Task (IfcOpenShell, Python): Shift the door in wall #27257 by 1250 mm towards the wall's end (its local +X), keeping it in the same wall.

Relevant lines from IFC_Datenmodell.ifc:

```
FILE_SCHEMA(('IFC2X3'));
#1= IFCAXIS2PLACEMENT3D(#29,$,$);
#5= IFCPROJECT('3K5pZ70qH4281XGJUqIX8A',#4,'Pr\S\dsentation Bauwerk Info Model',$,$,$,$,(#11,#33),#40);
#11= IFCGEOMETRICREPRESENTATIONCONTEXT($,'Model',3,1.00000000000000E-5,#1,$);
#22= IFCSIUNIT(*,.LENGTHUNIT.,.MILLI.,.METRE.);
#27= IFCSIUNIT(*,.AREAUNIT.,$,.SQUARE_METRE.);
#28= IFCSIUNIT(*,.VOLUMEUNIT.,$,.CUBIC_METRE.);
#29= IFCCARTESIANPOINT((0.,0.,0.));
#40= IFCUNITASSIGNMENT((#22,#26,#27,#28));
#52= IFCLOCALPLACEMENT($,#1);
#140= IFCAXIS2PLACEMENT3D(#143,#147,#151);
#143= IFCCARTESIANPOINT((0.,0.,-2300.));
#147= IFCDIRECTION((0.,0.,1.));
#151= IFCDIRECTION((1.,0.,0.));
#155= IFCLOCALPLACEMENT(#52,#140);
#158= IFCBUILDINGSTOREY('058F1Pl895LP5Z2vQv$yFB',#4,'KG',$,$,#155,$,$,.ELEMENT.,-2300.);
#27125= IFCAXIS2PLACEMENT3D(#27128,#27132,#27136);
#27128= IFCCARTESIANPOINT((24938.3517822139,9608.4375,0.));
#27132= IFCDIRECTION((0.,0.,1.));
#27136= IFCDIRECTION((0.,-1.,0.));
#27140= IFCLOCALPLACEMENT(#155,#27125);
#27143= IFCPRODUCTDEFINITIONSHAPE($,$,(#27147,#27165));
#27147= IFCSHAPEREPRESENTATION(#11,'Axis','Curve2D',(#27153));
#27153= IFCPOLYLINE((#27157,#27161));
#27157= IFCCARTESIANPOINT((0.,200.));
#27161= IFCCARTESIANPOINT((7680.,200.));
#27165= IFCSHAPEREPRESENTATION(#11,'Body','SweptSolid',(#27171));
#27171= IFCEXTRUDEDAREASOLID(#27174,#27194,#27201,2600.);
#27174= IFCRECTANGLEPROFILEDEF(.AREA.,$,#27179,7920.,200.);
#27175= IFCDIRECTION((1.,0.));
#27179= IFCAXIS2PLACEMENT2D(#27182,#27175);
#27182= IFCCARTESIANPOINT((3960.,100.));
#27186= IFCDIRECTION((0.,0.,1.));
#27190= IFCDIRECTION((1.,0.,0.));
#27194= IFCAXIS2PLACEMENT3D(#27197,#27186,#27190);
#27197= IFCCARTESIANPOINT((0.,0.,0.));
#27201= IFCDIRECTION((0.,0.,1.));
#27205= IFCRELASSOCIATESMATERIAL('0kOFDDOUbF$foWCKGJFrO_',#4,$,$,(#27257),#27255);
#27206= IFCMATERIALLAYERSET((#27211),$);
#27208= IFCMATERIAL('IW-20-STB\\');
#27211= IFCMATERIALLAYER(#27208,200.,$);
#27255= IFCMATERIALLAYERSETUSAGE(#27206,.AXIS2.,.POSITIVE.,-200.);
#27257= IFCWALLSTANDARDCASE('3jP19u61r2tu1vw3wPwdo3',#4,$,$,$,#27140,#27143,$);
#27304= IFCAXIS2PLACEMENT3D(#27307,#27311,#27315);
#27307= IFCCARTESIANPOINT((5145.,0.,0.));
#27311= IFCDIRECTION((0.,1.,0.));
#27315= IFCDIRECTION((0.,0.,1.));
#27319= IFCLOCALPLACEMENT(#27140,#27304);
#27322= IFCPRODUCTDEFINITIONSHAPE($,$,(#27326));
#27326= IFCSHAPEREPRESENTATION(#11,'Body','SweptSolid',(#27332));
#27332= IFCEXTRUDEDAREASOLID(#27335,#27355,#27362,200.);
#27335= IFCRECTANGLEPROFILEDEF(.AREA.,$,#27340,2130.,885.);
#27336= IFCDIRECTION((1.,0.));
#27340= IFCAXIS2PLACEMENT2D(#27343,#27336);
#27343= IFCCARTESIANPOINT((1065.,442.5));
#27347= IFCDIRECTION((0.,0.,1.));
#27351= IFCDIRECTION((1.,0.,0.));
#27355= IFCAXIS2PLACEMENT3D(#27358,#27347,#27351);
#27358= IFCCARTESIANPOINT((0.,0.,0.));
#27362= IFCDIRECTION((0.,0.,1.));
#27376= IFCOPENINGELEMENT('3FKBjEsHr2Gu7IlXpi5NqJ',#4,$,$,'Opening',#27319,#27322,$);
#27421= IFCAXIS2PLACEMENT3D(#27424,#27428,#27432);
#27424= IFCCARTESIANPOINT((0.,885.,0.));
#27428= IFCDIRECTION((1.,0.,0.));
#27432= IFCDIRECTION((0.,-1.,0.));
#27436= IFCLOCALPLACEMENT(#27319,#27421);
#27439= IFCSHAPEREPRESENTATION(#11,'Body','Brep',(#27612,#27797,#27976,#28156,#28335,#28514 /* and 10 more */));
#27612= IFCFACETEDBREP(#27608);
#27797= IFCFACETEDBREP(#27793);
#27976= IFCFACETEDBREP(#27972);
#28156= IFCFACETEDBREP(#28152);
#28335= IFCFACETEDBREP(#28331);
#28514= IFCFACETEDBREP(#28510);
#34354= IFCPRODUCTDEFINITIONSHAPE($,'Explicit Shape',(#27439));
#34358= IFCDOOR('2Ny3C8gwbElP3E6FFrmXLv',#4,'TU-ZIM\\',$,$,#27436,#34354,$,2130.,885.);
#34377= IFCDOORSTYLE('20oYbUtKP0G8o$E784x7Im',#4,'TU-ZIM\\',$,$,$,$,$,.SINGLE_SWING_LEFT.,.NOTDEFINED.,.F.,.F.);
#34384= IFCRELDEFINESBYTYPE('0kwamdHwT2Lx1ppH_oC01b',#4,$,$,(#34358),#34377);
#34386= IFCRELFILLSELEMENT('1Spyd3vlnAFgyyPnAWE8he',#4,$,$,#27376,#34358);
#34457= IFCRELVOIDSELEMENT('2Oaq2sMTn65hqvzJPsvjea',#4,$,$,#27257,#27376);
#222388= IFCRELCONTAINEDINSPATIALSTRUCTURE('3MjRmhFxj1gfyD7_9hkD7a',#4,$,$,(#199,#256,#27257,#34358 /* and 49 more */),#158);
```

```python
import ifcopenshell
import ifcopenshell.api.geometry
import ifcopenshell.util.placement
import ifcopenshell.util.unit

model = ifcopenshell.open("IFC_Datenmodell.ifc")
unit_scale = ifcopenshell.util.unit.calculate_unit_scale(model)

door = model.by_guid("2Ny3C8gwbElP3E6FFrmXLv")
opening = door.FillsVoids[0].RelatingOpeningElement
wall = opening.VoidsElements[0].RelatingBuildingElement

wall_matrix = ifcopenshell.util.placement.get_local_placement(wall.ObjectPlacement)
shift = wall_matrix[:3, 0] * 1.25 / unit_scale
before = ifcopenshell.util.placement.get_local_placement(door.ObjectPlacement)[:3, 3].copy()

# The door is placed relative to its opening, so it follows when the opening moves.
matrix = ifcopenshell.util.placement.get_local_placement(opening.ObjectPlacement)
matrix[:3, 3] += shift
ifcopenshell.api.geometry.edit_object_placement(
    model, product=opening, matrix=matrix, is_si=False, should_transform_children=True
)

after = ifcopenshell.util.placement.get_local_placement(door.ObjectPlacement)[:3, 3]
print("door moved by", (after - before).round(3) + 0.0)

model.write("IFC_Datenmodell_v2.ifc")
```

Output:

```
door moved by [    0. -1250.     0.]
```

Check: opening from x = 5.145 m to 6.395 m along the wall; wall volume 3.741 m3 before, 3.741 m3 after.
